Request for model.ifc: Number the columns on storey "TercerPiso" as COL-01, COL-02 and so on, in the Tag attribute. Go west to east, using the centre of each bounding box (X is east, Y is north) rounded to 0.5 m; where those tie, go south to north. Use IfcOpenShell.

First a look at what the model holds.

```python
import ifcopenshell
import ifcopenshell.util.element
import ifcopenshell.util.placement

model = ifcopenshell.open("model.ifc")
print(model.schema)
storey = next(s for s in model.by_type("IfcBuildingStorey") if s.Name == "TercerPiso")
columns = [e for e in ifcopenshell.util.element.get_decomposition(storey) if e.is_a("IfcColumn")]
for e in sorted(columns, key=lambda e: e.id()):
    origin = ifcopenshell.util.placement.get_local_placement(e.ObjectPlacement)[:3, 3]
    print(e.id(), e.Tag, e.Name, origin.round(2) + 0.0, sep=" | ")
```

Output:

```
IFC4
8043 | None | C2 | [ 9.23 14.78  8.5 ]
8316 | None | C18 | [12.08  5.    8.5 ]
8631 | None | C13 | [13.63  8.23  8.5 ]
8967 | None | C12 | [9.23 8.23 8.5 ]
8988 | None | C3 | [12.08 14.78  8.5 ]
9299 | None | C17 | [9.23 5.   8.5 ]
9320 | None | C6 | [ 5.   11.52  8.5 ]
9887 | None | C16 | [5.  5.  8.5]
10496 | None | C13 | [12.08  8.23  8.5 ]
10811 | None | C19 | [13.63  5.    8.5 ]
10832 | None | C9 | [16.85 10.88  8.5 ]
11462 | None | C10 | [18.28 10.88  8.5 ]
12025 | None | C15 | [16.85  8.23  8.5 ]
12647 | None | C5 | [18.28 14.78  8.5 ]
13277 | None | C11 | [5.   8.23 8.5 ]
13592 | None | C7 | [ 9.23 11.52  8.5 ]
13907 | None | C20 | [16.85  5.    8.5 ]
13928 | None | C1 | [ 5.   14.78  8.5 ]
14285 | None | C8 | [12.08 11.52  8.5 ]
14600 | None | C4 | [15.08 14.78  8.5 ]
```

```python
import ifcopenshell
import ifcopenshell.geom
import ifcopenshell.util.element
import ifcopenshell.util.shape

model = ifcopenshell.open("model.ifc")
settings = ifcopenshell.geom.settings()
settings.set("use-world-coords", True)


def centre(element):
    shape = ifcopenshell.geom.create_shape(settings, element)
    return ifcopenshell.util.shape.get_bbox_centroid(shape.geometry)


storey = next(s for s in model.by_type("IfcBuildingStorey") if s.Name == "TercerPiso")
columns = [e for e in ifcopenshell.util.element.get_decomposition(storey) if e.is_a("IfcColumn")]

# Insertion points can sit at a corner or the storey origin, so sort by the geometry (in metres).
centres = {e: centre(e) for e in columns}
columns.sort(key=lambda e: (round(centres[e][0] / 0.5), centres[e][1]))

for i, e in enumerate(columns, start=1):
    number = f"COL-{i:02d}"
    e.Tag = number
    print(e.id(), number)

model.write("model_v2.ifc")
```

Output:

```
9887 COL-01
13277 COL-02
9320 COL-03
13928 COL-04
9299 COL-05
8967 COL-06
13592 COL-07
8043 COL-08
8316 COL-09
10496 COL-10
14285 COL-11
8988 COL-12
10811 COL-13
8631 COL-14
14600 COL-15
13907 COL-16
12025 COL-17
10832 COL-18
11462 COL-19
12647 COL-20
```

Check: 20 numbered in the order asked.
